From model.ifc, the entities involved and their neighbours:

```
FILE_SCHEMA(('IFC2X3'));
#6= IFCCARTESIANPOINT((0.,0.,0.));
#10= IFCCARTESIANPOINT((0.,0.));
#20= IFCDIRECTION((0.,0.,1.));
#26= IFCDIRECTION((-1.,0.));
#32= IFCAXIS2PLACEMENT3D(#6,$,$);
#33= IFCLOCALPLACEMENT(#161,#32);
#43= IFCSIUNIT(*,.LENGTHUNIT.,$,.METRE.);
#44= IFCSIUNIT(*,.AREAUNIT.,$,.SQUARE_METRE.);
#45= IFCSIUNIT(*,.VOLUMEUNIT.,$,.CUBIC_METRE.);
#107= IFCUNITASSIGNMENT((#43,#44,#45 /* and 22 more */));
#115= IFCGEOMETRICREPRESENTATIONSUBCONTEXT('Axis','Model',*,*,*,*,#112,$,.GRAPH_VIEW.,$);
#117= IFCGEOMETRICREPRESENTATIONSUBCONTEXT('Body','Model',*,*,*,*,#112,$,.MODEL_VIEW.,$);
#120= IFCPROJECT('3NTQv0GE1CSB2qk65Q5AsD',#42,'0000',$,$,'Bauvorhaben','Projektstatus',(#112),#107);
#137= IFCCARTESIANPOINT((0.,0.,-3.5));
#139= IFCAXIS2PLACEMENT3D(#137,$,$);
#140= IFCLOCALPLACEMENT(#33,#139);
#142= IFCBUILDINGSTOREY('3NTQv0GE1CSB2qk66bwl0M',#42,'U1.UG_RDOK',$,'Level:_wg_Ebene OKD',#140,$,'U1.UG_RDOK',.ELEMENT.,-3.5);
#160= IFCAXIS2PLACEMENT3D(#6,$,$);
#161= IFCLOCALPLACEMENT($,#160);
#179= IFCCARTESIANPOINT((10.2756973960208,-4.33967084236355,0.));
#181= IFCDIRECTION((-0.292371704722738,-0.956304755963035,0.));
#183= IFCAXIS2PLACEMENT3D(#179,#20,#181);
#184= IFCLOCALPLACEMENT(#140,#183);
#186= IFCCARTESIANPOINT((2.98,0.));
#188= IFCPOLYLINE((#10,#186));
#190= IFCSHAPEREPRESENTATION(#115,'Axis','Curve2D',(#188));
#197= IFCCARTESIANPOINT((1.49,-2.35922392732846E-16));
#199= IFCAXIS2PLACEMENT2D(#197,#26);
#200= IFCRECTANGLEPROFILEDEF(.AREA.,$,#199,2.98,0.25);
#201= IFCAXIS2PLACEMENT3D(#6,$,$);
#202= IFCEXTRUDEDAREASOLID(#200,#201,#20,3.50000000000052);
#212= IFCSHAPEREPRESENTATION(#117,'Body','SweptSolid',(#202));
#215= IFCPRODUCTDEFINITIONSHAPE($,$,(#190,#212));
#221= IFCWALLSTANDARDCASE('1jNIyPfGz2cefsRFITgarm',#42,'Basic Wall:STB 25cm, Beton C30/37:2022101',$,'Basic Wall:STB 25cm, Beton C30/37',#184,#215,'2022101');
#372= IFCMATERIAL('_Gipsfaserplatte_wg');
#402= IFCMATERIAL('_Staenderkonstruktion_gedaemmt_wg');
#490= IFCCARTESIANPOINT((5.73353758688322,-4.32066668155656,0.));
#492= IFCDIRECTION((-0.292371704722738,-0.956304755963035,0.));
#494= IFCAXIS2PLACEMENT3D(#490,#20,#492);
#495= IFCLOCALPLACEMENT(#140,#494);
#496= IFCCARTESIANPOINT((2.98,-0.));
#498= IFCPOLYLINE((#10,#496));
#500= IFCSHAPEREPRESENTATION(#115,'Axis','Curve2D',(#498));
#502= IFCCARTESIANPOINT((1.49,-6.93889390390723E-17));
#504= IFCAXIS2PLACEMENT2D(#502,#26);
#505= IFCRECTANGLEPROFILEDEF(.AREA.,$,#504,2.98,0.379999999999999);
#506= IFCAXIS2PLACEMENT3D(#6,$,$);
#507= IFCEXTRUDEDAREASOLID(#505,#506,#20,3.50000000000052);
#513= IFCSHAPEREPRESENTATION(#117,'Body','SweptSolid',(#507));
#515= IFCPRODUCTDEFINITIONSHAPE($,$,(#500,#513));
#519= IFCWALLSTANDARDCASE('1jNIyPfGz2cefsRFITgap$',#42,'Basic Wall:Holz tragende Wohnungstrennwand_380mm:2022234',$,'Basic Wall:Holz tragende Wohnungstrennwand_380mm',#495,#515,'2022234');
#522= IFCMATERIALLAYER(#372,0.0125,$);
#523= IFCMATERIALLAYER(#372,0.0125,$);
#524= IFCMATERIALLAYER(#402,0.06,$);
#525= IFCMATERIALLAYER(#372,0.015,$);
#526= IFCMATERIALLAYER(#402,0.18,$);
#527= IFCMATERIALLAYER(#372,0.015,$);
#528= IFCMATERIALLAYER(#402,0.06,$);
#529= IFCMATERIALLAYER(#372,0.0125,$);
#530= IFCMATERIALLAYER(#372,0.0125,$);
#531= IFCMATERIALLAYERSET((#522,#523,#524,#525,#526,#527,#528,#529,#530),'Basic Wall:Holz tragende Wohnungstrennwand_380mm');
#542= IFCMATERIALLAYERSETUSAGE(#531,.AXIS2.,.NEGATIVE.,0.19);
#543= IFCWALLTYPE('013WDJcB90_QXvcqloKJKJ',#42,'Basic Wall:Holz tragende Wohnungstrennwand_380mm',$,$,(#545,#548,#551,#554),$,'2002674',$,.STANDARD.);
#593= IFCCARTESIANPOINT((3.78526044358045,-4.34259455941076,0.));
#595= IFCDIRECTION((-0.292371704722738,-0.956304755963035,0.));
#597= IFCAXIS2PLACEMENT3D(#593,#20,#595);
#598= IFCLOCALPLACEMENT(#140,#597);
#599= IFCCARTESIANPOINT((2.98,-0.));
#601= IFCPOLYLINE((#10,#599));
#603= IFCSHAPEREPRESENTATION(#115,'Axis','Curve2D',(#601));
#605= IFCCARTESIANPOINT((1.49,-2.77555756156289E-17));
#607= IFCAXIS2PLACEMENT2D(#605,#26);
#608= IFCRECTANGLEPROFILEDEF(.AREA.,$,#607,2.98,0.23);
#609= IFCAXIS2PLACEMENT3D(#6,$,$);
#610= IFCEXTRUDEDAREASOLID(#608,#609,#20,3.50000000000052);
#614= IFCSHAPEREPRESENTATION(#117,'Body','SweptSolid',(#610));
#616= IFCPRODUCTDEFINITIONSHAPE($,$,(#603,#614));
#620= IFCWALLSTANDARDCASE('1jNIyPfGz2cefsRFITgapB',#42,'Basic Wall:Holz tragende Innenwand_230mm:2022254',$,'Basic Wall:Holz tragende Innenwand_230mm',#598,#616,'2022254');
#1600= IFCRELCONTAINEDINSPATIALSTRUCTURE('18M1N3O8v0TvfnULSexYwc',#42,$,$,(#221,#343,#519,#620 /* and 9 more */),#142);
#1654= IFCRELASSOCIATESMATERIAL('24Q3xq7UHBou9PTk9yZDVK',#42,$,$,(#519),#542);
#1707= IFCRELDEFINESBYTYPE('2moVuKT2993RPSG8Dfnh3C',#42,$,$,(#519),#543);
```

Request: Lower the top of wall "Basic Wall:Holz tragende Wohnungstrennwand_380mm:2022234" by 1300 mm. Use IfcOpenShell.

```python
import ifcopenshell
import ifcopenshell.geom
import ifcopenshell.util.representation
import ifcopenshell.util.shape
import ifcopenshell.util.unit

model = ifcopenshell.open("model.ifc")
unit_scale = ifcopenshell.util.unit.calculate_unit_scale(model)
settings = ifcopenshell.geom.settings()


def volume(element):
    """Net volume in cubic metres, openings subtracted."""
    shape = ifcopenshell.geom.create_shape(settings, element)
    return ifcopenshell.util.shape.get_volume(shape.geometry)


wall = model.by_guid("1jNIyPfGz2cefsRFITgap$")
before = volume(wall)

body = ifcopenshell.util.representation.get_representation(wall, "Model", "Body")
solid = body.Items[0]
old_height = solid.Depth
solid.Depth -= 1.3 / unit_scale
after = volume(wall)

print(f"height {old_height:g} -> {solid.Depth:g}, volume {before:.3f} -> {after:.3f} m3")

model.write("model_v2.ifc")
```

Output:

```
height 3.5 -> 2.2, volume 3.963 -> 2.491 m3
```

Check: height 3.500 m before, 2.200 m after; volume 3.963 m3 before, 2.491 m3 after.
